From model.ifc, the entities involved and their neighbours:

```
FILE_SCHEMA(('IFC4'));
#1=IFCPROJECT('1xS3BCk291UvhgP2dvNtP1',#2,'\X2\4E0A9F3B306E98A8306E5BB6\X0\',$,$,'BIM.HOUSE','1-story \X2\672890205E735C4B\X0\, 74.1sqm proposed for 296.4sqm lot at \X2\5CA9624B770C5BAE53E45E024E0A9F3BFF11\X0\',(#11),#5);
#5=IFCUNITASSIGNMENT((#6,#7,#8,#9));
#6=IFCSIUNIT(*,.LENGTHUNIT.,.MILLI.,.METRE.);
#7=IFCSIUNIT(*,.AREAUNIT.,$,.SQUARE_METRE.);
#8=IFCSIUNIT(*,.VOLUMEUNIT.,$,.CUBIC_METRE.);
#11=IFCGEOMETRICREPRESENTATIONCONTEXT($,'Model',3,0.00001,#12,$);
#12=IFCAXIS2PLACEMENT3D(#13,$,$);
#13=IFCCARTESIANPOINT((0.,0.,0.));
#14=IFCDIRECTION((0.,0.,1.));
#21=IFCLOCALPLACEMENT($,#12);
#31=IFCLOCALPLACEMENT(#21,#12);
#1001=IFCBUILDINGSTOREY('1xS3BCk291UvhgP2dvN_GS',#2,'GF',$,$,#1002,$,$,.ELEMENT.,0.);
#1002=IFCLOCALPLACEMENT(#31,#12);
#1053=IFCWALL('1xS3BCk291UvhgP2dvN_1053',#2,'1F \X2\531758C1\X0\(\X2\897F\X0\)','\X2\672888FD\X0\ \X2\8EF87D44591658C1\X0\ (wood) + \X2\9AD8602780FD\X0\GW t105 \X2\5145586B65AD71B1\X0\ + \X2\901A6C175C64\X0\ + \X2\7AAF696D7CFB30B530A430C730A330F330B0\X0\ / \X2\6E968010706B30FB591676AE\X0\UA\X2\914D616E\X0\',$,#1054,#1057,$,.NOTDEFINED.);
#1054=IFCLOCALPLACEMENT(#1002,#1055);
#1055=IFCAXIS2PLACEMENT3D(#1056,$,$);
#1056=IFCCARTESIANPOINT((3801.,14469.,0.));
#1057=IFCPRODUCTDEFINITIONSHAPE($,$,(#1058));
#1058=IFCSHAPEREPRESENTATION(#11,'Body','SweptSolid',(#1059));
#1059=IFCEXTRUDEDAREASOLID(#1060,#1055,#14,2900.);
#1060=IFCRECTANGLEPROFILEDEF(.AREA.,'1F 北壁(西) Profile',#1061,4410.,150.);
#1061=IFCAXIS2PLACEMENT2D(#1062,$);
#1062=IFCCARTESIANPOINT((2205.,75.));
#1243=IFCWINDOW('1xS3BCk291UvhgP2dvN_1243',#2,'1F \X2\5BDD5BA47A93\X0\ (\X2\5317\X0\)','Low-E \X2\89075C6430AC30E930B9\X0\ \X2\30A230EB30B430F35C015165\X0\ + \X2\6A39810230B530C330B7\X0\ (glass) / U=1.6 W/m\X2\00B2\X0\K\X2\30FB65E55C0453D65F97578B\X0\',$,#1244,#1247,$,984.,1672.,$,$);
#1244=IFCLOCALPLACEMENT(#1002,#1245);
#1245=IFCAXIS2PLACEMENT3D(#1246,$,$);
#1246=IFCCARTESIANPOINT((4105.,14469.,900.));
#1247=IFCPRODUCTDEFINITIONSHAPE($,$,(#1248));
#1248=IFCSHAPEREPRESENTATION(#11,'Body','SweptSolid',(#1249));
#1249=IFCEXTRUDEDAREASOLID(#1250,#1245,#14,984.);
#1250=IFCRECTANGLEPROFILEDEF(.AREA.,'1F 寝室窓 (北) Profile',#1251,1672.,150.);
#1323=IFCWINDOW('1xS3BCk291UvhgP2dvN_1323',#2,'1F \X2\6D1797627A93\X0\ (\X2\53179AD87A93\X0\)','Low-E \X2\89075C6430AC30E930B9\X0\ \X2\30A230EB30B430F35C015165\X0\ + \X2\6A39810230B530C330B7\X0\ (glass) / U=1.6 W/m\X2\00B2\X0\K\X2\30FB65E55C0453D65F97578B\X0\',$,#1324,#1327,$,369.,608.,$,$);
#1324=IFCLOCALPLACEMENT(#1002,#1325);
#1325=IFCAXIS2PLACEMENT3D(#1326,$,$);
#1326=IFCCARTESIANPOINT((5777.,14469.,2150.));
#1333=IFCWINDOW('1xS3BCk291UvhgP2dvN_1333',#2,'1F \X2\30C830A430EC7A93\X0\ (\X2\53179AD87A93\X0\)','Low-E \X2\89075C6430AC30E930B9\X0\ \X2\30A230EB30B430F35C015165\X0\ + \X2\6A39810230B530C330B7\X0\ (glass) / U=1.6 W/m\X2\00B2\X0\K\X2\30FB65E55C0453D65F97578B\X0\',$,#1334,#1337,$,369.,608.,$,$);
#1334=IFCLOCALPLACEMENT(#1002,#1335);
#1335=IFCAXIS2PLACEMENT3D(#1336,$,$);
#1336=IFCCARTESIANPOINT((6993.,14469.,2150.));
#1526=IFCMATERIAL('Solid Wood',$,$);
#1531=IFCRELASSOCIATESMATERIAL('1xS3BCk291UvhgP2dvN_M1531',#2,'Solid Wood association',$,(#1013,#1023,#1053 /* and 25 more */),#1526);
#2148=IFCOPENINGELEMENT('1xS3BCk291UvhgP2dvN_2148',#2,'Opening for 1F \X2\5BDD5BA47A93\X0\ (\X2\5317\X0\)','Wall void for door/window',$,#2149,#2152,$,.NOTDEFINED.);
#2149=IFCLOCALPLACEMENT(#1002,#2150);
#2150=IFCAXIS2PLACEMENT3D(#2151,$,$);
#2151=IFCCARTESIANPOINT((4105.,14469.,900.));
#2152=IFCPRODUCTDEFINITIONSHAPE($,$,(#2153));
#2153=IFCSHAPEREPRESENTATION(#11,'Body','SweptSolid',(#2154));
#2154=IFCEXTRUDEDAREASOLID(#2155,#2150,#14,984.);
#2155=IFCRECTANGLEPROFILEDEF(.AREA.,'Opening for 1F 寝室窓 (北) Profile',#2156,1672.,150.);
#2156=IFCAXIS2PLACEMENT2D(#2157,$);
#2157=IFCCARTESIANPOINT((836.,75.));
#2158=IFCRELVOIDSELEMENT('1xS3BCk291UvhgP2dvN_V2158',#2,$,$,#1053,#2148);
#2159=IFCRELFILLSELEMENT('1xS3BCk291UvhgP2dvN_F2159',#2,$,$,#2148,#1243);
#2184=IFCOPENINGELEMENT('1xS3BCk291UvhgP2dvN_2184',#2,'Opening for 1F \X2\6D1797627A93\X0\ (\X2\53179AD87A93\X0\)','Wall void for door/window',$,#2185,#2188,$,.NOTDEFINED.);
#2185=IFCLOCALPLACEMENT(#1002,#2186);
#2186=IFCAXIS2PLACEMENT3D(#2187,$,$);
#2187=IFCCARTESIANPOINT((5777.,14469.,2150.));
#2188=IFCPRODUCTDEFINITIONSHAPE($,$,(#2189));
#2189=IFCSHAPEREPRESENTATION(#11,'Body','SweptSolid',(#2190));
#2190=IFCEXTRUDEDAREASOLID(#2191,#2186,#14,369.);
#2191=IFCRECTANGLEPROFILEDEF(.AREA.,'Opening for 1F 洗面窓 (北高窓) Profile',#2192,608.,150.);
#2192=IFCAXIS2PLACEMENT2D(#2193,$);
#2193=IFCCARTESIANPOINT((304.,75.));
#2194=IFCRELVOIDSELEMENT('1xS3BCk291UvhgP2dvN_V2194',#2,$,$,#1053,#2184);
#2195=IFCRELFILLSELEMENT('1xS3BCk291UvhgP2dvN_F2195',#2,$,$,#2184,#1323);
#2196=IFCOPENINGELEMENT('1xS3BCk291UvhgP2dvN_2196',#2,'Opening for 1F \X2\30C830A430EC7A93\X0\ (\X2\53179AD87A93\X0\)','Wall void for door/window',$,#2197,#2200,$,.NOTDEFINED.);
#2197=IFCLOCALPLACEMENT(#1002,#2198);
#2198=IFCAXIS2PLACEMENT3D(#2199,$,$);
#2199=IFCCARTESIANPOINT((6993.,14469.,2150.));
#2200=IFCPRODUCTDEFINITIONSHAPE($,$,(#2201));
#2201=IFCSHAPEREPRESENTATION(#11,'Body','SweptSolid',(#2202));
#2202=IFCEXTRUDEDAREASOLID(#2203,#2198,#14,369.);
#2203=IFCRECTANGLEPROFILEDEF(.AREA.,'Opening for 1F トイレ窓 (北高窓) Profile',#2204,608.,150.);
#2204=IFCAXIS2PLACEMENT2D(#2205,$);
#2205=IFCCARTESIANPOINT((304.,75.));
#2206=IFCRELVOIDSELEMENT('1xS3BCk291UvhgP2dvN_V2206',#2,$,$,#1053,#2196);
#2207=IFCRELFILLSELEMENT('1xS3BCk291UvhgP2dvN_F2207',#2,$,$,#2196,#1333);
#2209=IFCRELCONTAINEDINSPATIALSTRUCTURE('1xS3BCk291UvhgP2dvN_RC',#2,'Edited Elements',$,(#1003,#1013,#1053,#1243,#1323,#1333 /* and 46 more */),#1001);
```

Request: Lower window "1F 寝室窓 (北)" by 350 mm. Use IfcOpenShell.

```python
import numpy as np
import ifcopenshell
import ifcopenshell.api.geometry
import ifcopenshell.util.placement
import ifcopenshell.util.unit

model = ifcopenshell.open("model.ifc")
unit_scale = ifcopenshell.util.unit.calculate_unit_scale(model)

window = model.by_guid("1xS3BCk291UvhgP2dvN_1243")
opening = window.FillsVoids[0].RelatingOpeningElement
dz = -0.35 / unit_scale

shift = np.array([0.0, 0.0, dz])
# The window is not placed relative to its opening, so move both.
for product in (opening, window):
    matrix = ifcopenshell.util.placement.get_local_placement(product.ObjectPlacement)
    matrix[:3, 3] += shift
    ifcopenshell.api.geometry.edit_object_placement(model, product=product, matrix=matrix, is_si=False)

print(f"moved by {dz * unit_scale:+.3f} m")

model.write("model_v2.ifc")
```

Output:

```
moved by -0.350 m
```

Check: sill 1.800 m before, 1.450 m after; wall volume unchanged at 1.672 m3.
